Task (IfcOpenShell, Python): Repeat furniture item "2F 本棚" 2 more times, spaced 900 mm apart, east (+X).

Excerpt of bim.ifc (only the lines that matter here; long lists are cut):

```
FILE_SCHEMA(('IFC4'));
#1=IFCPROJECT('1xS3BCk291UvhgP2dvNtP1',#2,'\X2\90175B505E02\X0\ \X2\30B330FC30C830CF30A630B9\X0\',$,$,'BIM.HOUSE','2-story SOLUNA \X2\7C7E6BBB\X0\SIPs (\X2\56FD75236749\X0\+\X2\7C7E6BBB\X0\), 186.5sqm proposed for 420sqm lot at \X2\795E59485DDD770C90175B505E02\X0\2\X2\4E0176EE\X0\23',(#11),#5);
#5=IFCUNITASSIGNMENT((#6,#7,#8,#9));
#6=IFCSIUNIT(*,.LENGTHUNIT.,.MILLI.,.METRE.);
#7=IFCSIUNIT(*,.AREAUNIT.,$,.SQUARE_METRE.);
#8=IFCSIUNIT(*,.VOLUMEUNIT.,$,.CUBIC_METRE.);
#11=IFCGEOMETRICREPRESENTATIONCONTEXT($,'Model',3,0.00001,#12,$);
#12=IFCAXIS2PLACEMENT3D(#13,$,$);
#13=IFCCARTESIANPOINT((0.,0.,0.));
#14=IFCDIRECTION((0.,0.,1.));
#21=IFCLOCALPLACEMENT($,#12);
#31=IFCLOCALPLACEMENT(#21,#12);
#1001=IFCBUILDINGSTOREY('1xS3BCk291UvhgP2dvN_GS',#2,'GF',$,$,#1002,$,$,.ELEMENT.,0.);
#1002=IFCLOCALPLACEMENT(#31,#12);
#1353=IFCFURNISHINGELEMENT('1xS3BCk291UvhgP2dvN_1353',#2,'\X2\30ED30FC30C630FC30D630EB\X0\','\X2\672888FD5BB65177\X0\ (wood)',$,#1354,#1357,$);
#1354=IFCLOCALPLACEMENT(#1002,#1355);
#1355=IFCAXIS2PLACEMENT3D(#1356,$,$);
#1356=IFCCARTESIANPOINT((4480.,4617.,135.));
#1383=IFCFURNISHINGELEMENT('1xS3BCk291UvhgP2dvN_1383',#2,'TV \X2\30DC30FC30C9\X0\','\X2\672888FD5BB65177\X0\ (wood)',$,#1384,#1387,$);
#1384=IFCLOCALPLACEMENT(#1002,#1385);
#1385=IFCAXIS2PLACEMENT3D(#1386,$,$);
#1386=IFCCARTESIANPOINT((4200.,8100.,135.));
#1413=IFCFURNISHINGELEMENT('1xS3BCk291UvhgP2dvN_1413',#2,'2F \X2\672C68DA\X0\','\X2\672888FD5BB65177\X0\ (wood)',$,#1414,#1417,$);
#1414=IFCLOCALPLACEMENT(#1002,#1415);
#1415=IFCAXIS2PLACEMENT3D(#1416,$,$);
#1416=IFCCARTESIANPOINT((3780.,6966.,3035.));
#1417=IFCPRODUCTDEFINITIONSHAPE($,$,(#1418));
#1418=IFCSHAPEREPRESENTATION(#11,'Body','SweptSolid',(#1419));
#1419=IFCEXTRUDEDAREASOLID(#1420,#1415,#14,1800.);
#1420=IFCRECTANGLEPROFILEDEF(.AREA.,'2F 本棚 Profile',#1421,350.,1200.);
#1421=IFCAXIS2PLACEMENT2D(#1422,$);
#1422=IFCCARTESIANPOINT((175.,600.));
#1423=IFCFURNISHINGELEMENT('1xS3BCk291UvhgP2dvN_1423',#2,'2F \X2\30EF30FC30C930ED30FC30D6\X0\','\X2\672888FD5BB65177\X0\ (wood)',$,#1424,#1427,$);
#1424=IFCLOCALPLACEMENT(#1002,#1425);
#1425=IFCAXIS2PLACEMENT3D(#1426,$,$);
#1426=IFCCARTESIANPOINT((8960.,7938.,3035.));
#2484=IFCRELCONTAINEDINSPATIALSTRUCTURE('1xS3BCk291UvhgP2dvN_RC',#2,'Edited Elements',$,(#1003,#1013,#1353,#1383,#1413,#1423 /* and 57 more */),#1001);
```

```python
import numpy as np
import ifcopenshell
import ifcopenshell.api.geometry
import ifcopenshell.api.root
import ifcopenshell.util.element
import ifcopenshell.util.placement
import ifcopenshell.util.unit

model = ifcopenshell.open("bim.ifc")
unit_scale = ifcopenshell.util.unit.calculate_unit_scale(model)


def reuse_history(source, copy):
    """copy_class also copies each property set's owner history, people and application; keep the originals."""
    for rel in copy.IsDefinedBy:
        if rel.is_a("IfcRelDefinesByProperties") and (history := rel.RelatingPropertyDefinition.OwnerHistory):
            rel.RelatingPropertyDefinition.OwnerHistory = source.OwnerHistory
            ifcopenshell.util.element.remove_deep2(model, history)


source = model.by_guid("1xS3BCk291UvhgP2dvN_1413")
base = ifcopenshell.util.placement.get_local_placement(source.ObjectPlacement)
step = np.array([1.0, 0.0, 0.0]) * 0.9 / unit_scale

for i in range(1, 3):
    copy = ifcopenshell.api.root.copy_class(model, product=source)
    copy.Representation = ifcopenshell.util.element.copy_deep(
        model, source.Representation, exclude=["IfcGeometricRepresentationContext", "IfcRepresentationMap"]
    )
    reuse_history(source, copy)
    matrix = base.copy()
    matrix[:3, 3] += i * step
    print("added at", matrix[:3, 3].round(3) + 0.0)
    ifcopenshell.api.geometry.edit_object_placement(model, product=copy, matrix=matrix, is_si=False)

model.write("bim_v2.ifc")
```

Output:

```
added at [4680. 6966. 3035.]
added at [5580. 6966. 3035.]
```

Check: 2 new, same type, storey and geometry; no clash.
